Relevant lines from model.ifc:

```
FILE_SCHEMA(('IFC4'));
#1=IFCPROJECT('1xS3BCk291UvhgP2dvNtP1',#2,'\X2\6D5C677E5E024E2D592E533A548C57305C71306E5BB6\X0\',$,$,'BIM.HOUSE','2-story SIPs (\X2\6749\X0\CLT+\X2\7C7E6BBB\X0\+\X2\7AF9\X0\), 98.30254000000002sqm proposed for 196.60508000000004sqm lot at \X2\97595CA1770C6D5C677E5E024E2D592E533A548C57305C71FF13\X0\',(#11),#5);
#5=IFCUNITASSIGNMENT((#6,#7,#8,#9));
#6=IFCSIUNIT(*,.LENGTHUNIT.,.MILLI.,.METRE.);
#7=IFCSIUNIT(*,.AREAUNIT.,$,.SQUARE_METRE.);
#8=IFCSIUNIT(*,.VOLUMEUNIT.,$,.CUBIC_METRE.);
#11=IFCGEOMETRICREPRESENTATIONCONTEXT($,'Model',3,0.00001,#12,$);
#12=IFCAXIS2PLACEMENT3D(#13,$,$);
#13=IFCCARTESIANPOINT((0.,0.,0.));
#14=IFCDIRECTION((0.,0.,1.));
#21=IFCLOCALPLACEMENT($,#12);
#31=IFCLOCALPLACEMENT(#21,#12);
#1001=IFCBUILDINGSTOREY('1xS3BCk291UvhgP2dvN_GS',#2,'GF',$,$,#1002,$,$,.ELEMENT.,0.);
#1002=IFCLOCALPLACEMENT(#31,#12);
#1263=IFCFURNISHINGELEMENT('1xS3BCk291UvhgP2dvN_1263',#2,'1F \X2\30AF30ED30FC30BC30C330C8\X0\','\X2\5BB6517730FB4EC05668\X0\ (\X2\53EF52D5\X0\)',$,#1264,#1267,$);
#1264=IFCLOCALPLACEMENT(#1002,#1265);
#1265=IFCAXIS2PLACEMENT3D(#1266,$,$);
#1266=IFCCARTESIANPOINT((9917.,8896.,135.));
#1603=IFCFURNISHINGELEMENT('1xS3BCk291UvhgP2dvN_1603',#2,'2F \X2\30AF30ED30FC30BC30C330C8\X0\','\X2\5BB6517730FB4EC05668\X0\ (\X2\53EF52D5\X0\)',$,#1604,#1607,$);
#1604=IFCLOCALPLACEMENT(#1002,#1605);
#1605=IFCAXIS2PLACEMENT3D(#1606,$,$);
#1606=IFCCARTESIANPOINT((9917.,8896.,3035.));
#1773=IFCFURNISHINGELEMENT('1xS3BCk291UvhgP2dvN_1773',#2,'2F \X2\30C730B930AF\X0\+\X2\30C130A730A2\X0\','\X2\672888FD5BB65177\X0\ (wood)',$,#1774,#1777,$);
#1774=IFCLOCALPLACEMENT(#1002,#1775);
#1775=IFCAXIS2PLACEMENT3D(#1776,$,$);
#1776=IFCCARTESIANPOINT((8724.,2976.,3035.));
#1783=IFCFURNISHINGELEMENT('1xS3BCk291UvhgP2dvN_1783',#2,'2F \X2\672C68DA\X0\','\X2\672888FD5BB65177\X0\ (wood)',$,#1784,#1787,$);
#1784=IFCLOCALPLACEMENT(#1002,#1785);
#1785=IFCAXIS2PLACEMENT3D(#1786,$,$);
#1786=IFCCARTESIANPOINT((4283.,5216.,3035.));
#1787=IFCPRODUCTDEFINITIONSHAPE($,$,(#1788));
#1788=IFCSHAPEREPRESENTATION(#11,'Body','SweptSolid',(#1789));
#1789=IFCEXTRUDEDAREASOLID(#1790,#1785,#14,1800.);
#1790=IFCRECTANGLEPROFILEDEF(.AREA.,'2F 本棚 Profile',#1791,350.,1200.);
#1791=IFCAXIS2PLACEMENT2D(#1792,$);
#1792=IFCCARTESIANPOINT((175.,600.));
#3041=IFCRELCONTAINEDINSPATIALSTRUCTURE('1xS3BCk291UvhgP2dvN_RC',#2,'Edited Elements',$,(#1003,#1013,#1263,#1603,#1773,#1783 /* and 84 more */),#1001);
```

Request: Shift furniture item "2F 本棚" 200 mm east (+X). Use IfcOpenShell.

```python
import ifcopenshell
import ifcopenshell.api.geometry
import ifcopenshell.util.placement
import ifcopenshell.util.unit

model = ifcopenshell.open("model.ifc")
unit_scale = ifcopenshell.util.unit.calculate_unit_scale(model)

item = model.by_guid("1xS3BCk291UvhgP2dvN_1783")
matrix = ifcopenshell.util.placement.get_local_placement(item.ObjectPlacement)
matrix[0, 3] += 0.2 / unit_scale
ifcopenshell.api.geometry.edit_object_placement(model, product=item, matrix=matrix, is_si=False)

print(ifcopenshell.util.placement.get_local_placement(item.ObjectPlacement).round(3) + 0.0)

model.write("model_v2.ifc")
```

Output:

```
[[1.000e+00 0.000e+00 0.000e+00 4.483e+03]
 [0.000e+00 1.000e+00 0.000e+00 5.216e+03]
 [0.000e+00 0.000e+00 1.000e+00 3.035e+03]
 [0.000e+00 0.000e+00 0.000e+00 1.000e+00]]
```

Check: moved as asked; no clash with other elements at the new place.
